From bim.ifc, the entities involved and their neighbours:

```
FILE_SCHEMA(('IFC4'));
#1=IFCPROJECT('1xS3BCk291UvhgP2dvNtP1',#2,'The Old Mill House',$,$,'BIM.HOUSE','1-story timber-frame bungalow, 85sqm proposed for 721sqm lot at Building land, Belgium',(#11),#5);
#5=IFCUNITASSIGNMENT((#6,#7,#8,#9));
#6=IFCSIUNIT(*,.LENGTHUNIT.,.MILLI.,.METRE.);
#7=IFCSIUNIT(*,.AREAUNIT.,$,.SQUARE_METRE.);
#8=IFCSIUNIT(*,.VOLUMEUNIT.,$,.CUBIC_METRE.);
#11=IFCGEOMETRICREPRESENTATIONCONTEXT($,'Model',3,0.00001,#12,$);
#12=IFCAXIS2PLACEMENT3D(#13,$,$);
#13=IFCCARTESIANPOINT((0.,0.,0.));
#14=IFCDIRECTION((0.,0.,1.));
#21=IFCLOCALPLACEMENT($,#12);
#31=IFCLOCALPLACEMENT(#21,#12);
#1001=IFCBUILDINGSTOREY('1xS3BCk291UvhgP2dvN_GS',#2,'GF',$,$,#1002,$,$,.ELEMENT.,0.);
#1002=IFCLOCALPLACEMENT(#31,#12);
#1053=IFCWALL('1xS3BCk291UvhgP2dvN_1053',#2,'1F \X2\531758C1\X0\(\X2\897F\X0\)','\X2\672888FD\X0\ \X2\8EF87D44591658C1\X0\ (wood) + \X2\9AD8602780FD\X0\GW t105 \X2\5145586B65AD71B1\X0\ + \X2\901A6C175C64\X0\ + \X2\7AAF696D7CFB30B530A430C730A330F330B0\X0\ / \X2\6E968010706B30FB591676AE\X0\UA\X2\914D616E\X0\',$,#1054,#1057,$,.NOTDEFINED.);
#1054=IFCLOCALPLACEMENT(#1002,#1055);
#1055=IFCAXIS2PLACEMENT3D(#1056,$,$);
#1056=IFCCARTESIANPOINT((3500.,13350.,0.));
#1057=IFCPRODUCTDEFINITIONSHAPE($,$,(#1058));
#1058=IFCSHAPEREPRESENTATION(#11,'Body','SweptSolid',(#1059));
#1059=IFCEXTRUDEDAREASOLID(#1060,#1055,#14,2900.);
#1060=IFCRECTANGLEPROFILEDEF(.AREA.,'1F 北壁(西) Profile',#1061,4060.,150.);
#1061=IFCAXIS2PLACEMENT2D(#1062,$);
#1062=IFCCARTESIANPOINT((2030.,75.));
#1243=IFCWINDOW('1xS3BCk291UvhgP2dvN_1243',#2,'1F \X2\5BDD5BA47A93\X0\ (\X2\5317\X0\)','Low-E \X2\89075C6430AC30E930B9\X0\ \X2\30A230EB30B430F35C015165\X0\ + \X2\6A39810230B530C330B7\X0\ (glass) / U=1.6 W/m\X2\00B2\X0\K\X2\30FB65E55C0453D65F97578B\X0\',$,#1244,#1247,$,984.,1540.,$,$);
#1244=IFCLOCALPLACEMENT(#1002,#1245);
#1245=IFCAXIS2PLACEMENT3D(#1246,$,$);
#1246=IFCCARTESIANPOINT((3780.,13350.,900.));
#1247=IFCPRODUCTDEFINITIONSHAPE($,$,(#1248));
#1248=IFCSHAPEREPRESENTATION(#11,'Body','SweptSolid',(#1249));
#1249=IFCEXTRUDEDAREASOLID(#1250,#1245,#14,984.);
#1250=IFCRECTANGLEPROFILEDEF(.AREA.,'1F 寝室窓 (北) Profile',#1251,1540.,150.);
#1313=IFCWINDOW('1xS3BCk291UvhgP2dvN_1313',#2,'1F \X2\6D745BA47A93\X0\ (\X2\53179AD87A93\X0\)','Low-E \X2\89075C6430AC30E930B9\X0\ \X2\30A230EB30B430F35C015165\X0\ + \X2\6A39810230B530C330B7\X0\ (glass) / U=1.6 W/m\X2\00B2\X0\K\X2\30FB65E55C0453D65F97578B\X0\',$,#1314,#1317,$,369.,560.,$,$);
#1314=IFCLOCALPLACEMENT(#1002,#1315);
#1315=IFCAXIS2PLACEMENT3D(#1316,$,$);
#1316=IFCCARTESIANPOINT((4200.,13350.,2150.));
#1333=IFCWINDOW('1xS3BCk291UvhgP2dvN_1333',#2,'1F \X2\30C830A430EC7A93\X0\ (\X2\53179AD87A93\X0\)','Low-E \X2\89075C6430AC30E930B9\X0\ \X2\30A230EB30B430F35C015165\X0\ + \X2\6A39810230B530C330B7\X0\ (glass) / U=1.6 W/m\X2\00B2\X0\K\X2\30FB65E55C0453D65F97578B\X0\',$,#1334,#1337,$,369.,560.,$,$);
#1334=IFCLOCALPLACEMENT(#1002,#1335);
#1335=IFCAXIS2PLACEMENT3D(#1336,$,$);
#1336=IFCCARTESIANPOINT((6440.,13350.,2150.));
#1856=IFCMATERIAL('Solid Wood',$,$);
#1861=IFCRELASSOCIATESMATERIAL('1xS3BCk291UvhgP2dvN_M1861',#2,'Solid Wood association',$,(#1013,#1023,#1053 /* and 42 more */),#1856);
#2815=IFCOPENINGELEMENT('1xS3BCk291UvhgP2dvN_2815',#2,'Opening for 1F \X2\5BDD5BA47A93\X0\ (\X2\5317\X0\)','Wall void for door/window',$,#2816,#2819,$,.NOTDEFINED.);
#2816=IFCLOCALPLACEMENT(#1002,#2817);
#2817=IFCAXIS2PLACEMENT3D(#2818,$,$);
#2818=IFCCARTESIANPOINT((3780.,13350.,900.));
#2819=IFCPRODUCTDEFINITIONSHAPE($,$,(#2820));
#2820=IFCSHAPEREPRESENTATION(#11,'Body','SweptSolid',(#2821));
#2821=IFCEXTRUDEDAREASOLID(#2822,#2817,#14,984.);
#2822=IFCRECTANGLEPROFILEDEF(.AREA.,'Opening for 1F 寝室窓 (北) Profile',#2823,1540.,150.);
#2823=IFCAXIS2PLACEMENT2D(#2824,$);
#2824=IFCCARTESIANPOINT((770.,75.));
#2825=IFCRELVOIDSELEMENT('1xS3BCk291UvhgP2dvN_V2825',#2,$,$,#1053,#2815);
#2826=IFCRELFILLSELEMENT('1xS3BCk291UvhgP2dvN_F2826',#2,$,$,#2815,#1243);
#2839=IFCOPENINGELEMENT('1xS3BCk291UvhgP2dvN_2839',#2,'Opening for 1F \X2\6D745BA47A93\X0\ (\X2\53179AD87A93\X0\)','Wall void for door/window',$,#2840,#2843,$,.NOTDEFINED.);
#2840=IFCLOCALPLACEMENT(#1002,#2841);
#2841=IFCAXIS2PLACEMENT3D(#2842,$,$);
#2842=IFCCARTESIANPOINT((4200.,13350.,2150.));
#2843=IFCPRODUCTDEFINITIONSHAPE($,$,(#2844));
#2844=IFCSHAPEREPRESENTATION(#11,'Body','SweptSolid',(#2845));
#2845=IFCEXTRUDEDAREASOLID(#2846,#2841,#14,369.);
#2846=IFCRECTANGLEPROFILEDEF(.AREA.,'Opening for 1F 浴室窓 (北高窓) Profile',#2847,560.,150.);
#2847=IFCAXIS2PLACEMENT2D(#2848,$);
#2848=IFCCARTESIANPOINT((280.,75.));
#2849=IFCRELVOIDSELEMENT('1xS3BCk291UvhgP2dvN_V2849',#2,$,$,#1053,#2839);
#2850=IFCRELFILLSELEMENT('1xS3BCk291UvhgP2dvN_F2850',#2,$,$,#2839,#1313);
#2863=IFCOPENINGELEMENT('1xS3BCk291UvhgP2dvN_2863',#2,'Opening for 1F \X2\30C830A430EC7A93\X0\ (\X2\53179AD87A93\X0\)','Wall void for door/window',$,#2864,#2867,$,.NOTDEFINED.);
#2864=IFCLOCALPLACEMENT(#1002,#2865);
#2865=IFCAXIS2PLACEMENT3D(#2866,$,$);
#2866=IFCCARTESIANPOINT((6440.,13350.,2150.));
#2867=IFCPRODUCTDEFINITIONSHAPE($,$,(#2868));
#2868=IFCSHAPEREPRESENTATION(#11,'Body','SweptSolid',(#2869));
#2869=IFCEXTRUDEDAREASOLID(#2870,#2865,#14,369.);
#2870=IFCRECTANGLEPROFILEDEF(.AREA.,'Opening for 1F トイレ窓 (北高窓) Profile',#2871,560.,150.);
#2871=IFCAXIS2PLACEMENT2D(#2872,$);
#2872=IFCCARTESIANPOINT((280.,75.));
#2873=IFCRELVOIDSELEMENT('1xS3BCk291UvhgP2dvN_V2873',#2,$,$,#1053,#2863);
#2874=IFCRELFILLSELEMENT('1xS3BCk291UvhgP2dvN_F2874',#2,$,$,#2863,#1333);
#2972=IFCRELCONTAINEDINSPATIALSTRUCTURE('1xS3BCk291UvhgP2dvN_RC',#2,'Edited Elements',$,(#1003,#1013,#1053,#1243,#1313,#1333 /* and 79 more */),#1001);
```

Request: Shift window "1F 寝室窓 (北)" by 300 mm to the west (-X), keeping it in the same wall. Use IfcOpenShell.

```python
import ifcopenshell
import ifcopenshell.api.geometry
import ifcopenshell.util.placement
import ifcopenshell.util.unit

model = ifcopenshell.open("bim.ifc")
unit_scale = ifcopenshell.util.unit.calculate_unit_scale(model)

window = model.by_guid("1xS3BCk291UvhgP2dvN_1243")
opening = window.FillsVoids[0].RelatingOpeningElement
wall = opening.VoidsElements[0].RelatingBuildingElement

wall_matrix = ifcopenshell.util.placement.get_local_placement(wall.ObjectPlacement)
shift = wall_matrix[:3, 0] * -0.3 / unit_scale
before = ifcopenshell.util.placement.get_local_placement(window.ObjectPlacement)[:3, 3].copy()

# The window is not placed relative to its opening, so move both.
for product in (opening, window):
    matrix = ifcopenshell.util.placement.get_local_placement(product.ObjectPlacement)
    matrix[:3, 3] += shift
    ifcopenshell.api.geometry.edit_object_placement(model, product=product, matrix=matrix, is_si=False)

after = ifcopenshell.util.placement.get_local_placement(window.ObjectPlacement)[:3, 3]
print("window moved by", (after - before).round(3) + 0.0)

model.write("bim_edited.ifc")
```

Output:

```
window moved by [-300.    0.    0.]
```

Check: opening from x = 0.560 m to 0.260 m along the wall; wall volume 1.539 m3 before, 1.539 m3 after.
